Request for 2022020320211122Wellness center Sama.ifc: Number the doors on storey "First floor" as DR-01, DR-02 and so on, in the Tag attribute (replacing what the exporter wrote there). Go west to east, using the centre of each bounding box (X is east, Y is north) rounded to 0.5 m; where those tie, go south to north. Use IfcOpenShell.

First a look at what the model holds.

```python
import ifcopenshell
import ifcopenshell.util.element
import ifcopenshell.util.placement

model = ifcopenshell.open("2022020320211122Wellness center Sama.ifc")
print(model.schema)
storey = next(s for s in model.by_type("IfcBuildingStorey") if s.Name == "First floor")
doors = [e for e in ifcopenshell.util.element.get_decomposition(storey) if e.is_a("IfcDoor")]
for e in sorted(doors, key=lambda e: e.id()):
    origin = ifcopenshell.util.placement.get_local_placement(e.ObjectPlacement)[:3, 3]
    print(e.id(), e.Tag, e.Name, origin.round(2) + 0.0, sep=" | ")
```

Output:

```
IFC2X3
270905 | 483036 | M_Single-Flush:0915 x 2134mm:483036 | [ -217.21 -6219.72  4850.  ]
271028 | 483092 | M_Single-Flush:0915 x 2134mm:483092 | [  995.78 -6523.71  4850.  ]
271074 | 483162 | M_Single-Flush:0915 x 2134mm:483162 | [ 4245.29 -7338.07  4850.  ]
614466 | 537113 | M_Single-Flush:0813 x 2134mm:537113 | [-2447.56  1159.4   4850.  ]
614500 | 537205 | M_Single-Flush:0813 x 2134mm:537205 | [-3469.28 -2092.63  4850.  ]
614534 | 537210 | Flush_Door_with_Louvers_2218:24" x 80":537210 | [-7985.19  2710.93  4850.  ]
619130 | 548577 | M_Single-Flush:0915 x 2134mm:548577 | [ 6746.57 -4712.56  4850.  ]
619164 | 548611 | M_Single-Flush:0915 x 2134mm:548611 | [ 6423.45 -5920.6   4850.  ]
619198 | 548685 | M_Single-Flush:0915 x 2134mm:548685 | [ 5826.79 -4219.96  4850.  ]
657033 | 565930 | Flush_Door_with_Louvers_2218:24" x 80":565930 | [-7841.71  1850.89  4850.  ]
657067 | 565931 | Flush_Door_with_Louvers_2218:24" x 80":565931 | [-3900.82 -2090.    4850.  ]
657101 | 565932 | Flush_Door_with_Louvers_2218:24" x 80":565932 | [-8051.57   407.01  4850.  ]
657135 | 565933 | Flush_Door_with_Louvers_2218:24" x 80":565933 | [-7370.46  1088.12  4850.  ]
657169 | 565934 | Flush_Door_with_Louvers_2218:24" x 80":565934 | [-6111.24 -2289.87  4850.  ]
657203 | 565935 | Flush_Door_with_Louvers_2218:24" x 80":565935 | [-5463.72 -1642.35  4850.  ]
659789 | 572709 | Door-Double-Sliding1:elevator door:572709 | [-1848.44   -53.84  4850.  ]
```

```python
import ifcopenshell
import ifcopenshell.geom
import ifcopenshell.util.element
import ifcopenshell.util.shape

model = ifcopenshell.open("2022020320211122Wellness center Sama.ifc")
settings = ifcopenshell.geom.settings()
settings.set("use-world-coords", True)


def centre(element):
    shape = ifcopenshell.geom.create_shape(settings, element)
    return ifcopenshell.util.shape.get_bbox_centroid(shape.geometry)


storey = next(s for s in model.by_type("IfcBuildingStorey") if s.Name == "First floor")
doors = [e for e in ifcopenshell.util.element.get_decomposition(storey) if e.is_a("IfcDoor")]

# Insertion points can sit at a corner or the storey origin, so sort by the geometry (in metres).
centres = {e: centre(e) for e in doors}
doors.sort(key=lambda e: (round(centres[e][0] / 0.5), centres[e][1]))

for i, e in enumerate(doors, start=1):
    number = f"DR-{i:02d}"
    e.Tag = number
    print(e.id(), number)

model.write("2022020320211122Wellness center Sama-out.ifc")
```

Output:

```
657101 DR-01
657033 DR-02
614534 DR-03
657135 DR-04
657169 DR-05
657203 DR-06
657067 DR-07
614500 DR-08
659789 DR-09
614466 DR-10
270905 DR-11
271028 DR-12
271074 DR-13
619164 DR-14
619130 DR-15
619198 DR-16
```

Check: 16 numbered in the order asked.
